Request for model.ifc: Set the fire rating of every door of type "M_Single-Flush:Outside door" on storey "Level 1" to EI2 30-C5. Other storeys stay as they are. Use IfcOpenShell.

First a look at what the model holds.

```python
import ifcopenshell
import ifcopenshell.util.element

model = ifcopenshell.open("model.ifc")
print(model.schema)
storey = next(s for s in model.by_type("IfcBuildingStorey") if s.Name == "Level 1")
doors = [e for e in ifcopenshell.util.element.get_decomposition(storey) if e.is_a("IfcDoor")]
seen = {}
for e in doors:
    element_type = ifcopenshell.util.element.get_type(e)
    key = (element_type.Name if element_type != e and element_type else None, ifcopenshell.util.element.get_pset(e, "Pset_DoorCommon", "FireRating"))
    seen[key] = seen.get(key, 0) + 1
for (name, value), count in sorted(seen.items(), key=str):
    print(count, "x", name, "|", value)
```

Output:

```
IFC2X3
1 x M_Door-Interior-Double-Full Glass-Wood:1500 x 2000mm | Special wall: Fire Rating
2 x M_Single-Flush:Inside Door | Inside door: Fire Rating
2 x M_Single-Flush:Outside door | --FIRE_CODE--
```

```python
import ifcopenshell
import ifcopenshell.api.pset
import ifcopenshell.util.element

model = ifcopenshell.open("model.ifc")

storey = next(s for s in model.by_type("IfcBuildingStorey") if s.Name == "Level 1")
doors = [e for e in ifcopenshell.util.element.get_decomposition(storey) if e.is_a("IfcDoor")]

count = 0
for e in doors:
    element_type = ifcopenshell.util.element.get_type(e)
    if element_type in (None, e) or element_type.Name != "M_Single-Flush:Outside door":
        continue
    # add_pset returns the element's existing set when there is one.
    pset = ifcopenshell.api.pset.add_pset(model, product=e, name="Pset_DoorCommon")
    ifcopenshell.api.pset.edit_pset(model, pset=pset, properties={"FireRating": "EI2 30-C5"})
    count += 1

print(count, "doors updated")

model.write("model_edited.ifc")
```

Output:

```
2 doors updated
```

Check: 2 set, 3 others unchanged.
